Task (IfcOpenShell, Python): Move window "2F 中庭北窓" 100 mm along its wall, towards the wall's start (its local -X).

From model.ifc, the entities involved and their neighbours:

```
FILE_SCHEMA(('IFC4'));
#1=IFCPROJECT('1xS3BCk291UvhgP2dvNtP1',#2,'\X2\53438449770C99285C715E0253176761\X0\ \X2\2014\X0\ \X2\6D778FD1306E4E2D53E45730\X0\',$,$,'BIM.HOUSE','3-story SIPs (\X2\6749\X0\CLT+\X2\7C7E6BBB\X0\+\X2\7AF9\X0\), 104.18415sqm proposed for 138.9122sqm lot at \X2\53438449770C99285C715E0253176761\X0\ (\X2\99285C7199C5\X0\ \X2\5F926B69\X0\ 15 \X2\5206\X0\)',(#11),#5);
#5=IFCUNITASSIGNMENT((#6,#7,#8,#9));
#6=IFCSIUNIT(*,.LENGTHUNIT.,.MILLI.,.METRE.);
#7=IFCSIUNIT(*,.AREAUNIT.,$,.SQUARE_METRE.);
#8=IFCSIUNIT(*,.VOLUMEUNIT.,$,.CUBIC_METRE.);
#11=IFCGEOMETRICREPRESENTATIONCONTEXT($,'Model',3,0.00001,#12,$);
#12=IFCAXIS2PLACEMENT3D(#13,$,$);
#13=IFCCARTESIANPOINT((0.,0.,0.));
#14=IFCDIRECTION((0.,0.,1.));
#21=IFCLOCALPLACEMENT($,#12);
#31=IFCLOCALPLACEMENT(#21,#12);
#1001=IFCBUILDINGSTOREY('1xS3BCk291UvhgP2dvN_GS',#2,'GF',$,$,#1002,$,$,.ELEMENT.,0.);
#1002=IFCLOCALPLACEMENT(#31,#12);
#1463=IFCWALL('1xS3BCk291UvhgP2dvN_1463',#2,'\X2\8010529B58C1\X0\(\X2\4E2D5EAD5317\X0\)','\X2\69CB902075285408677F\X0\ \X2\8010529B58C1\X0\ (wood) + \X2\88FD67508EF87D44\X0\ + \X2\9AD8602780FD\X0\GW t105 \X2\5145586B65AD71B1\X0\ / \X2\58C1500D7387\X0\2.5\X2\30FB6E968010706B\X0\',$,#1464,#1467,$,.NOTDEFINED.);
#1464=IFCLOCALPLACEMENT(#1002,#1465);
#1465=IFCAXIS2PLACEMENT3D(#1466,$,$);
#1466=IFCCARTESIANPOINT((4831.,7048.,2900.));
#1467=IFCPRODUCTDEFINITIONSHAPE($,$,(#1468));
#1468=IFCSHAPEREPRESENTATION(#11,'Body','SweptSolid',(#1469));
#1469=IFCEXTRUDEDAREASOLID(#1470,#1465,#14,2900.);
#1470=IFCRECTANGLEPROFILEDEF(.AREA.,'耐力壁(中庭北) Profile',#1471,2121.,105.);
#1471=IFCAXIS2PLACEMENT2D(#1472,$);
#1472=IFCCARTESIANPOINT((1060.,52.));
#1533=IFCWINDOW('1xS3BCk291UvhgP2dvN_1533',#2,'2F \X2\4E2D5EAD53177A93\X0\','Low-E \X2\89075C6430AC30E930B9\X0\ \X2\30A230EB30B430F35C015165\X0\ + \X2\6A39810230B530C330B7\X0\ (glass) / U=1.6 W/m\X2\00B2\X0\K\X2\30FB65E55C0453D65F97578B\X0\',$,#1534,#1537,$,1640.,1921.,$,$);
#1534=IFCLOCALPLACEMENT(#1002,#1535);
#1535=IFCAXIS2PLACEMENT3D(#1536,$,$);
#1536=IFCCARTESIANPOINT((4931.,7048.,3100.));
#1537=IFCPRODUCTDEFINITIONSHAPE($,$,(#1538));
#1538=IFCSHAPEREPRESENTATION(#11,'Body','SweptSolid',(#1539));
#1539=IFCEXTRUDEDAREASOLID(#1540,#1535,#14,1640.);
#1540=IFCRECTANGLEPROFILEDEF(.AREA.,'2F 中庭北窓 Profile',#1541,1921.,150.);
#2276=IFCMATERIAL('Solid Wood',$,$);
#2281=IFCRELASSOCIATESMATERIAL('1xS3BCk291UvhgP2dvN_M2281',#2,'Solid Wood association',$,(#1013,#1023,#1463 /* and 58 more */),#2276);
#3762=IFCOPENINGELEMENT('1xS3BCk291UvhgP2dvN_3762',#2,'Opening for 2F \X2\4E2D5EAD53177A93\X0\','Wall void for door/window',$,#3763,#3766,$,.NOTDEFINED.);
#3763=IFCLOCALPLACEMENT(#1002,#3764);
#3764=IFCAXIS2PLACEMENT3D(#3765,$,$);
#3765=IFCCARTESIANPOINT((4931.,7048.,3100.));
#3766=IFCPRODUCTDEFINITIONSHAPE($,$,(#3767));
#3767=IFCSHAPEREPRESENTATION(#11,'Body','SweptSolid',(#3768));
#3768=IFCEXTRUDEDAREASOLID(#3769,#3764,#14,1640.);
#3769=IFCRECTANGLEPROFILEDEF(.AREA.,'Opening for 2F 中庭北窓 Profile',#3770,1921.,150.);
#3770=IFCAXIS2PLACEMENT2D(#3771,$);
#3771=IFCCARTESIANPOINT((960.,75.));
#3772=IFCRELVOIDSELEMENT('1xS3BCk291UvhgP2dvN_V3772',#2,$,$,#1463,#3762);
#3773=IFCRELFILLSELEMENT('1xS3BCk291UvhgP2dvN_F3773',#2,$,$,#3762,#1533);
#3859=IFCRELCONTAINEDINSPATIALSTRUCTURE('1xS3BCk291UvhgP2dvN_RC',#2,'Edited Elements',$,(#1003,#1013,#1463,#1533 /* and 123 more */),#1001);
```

```python
import ifcopenshell
import ifcopenshell.api.geometry
import ifcopenshell.util.placement

model = ifcopenshell.open("model.ifc")

window = model.by_id(1533)
opening = window.FillsVoids[0].RelatingOpeningElement
wall = opening.VoidsElements[0].RelatingBuildingElement

wall_matrix = ifcopenshell.util.placement.get_local_placement(wall.ObjectPlacement)
shift = wall_matrix[:3, 0] * -100.0
before = ifcopenshell.util.placement.get_local_placement(window.ObjectPlacement)[:3, 3].copy()

# The window is not placed relative to its opening, so move both.
for product in (opening, window):
    matrix = ifcopenshell.util.placement.get_local_placement(product.ObjectPlacement)
    matrix[:3, 3] += shift
    ifcopenshell.api.geometry.edit_object_placement(model, product=product, matrix=matrix, is_si=False)

after = ifcopenshell.util.placement.get_local_placement(window.ObjectPlacement)[:3, 3]
print("window moved by", (after - before).round(3) + 0.0)

model.write("model_v2.ifc")
```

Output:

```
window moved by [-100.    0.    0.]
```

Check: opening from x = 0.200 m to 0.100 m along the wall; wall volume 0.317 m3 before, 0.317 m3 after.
